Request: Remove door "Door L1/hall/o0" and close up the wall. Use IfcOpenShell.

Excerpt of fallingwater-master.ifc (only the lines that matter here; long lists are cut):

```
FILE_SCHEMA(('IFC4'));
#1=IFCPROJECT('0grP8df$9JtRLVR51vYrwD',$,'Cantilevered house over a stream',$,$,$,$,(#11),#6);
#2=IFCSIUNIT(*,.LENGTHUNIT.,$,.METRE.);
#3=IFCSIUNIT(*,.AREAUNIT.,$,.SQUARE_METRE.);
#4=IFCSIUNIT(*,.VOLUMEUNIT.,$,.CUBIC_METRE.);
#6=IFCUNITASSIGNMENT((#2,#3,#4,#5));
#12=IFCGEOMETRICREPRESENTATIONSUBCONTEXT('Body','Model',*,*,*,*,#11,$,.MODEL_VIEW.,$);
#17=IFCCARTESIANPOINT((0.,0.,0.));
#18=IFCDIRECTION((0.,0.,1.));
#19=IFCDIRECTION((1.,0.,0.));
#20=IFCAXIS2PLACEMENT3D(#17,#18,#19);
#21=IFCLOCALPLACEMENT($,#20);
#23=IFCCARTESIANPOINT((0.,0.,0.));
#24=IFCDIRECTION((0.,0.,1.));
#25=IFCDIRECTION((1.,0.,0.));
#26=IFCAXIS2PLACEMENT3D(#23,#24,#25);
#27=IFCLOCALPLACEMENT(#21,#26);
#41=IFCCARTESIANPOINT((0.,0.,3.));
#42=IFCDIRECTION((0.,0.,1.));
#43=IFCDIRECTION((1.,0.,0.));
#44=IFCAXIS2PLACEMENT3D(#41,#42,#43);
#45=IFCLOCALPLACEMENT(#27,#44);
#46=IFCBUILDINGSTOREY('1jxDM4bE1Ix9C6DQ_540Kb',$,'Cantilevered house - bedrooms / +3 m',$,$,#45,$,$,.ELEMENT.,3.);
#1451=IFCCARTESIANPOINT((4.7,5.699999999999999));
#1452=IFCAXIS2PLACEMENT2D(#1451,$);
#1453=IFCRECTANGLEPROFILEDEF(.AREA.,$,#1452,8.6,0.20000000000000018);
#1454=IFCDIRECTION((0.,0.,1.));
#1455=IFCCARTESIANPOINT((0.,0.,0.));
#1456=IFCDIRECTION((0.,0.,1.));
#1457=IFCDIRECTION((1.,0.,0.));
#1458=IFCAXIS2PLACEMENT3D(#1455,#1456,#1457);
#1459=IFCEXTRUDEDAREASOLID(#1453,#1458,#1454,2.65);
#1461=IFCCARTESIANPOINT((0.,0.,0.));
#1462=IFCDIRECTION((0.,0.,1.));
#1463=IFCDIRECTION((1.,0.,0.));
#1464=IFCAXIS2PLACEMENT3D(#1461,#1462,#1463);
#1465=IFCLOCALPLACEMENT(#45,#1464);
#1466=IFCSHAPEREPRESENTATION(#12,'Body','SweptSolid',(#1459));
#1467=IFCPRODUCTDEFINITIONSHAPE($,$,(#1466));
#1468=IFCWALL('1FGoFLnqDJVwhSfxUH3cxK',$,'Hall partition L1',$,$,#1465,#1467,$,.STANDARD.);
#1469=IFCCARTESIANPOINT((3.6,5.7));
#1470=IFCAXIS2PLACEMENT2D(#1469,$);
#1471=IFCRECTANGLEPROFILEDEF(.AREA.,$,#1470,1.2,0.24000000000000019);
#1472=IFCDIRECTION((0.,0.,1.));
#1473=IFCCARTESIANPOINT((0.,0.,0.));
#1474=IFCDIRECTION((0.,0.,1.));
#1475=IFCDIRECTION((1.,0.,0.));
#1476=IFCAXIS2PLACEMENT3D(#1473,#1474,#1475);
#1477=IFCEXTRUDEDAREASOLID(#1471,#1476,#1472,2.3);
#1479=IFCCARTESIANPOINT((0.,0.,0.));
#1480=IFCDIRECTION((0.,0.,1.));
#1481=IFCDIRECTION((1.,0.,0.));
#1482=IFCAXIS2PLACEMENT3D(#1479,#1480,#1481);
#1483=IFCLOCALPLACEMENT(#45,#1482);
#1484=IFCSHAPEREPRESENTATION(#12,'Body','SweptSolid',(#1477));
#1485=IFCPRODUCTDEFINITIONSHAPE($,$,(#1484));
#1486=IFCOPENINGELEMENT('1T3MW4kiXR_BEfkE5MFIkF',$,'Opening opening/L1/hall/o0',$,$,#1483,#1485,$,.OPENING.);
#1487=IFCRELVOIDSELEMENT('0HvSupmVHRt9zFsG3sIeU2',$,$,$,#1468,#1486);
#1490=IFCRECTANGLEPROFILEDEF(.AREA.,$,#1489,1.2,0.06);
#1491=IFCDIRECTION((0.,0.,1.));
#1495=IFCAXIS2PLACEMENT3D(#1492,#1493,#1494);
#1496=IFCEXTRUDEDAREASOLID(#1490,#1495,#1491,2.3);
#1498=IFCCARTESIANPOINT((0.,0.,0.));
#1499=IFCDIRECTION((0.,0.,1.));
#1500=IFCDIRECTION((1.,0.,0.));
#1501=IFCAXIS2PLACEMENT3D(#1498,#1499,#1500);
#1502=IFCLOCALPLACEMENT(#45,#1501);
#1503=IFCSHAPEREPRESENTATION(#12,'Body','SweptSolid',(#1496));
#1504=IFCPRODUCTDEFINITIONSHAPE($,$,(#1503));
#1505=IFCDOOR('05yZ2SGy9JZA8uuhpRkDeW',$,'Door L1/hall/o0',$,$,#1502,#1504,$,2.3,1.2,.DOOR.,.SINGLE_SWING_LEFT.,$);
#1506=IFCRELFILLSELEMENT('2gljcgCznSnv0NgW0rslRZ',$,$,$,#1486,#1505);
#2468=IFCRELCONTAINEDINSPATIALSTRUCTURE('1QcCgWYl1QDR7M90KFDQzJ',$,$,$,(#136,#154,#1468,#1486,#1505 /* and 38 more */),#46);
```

```python
import ifcopenshell
import ifcopenshell.api.feature
import ifcopenshell.api.root
import ifcopenshell.geom
import ifcopenshell.util.shape

model = ifcopenshell.open("fallingwater-master.ifc")
settings = ifcopenshell.geom.settings()


def volume(element):
    """Net volume in cubic metres, openings subtracted."""
    shape = ifcopenshell.geom.create_shape(settings, element)
    return ifcopenshell.util.shape.get_volume(shape.geometry)


door = model.by_id(1505)
opening = door.FillsVoids[0].RelatingOpeningElement
wall = opening.VoidsElements[0].RelatingBuildingElement
before = volume(wall)

ifcopenshell.api.root.remove_product(model, product=door)
ifcopenshell.api.feature.remove_feature(model, feature=opening)

after = volume(wall)

print(f"wall volume {before:.3f} -> {after:.3f} m3")

model.write("fallingwater-master_v2.ifc")
```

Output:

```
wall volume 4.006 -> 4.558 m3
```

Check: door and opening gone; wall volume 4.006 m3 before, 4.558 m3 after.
